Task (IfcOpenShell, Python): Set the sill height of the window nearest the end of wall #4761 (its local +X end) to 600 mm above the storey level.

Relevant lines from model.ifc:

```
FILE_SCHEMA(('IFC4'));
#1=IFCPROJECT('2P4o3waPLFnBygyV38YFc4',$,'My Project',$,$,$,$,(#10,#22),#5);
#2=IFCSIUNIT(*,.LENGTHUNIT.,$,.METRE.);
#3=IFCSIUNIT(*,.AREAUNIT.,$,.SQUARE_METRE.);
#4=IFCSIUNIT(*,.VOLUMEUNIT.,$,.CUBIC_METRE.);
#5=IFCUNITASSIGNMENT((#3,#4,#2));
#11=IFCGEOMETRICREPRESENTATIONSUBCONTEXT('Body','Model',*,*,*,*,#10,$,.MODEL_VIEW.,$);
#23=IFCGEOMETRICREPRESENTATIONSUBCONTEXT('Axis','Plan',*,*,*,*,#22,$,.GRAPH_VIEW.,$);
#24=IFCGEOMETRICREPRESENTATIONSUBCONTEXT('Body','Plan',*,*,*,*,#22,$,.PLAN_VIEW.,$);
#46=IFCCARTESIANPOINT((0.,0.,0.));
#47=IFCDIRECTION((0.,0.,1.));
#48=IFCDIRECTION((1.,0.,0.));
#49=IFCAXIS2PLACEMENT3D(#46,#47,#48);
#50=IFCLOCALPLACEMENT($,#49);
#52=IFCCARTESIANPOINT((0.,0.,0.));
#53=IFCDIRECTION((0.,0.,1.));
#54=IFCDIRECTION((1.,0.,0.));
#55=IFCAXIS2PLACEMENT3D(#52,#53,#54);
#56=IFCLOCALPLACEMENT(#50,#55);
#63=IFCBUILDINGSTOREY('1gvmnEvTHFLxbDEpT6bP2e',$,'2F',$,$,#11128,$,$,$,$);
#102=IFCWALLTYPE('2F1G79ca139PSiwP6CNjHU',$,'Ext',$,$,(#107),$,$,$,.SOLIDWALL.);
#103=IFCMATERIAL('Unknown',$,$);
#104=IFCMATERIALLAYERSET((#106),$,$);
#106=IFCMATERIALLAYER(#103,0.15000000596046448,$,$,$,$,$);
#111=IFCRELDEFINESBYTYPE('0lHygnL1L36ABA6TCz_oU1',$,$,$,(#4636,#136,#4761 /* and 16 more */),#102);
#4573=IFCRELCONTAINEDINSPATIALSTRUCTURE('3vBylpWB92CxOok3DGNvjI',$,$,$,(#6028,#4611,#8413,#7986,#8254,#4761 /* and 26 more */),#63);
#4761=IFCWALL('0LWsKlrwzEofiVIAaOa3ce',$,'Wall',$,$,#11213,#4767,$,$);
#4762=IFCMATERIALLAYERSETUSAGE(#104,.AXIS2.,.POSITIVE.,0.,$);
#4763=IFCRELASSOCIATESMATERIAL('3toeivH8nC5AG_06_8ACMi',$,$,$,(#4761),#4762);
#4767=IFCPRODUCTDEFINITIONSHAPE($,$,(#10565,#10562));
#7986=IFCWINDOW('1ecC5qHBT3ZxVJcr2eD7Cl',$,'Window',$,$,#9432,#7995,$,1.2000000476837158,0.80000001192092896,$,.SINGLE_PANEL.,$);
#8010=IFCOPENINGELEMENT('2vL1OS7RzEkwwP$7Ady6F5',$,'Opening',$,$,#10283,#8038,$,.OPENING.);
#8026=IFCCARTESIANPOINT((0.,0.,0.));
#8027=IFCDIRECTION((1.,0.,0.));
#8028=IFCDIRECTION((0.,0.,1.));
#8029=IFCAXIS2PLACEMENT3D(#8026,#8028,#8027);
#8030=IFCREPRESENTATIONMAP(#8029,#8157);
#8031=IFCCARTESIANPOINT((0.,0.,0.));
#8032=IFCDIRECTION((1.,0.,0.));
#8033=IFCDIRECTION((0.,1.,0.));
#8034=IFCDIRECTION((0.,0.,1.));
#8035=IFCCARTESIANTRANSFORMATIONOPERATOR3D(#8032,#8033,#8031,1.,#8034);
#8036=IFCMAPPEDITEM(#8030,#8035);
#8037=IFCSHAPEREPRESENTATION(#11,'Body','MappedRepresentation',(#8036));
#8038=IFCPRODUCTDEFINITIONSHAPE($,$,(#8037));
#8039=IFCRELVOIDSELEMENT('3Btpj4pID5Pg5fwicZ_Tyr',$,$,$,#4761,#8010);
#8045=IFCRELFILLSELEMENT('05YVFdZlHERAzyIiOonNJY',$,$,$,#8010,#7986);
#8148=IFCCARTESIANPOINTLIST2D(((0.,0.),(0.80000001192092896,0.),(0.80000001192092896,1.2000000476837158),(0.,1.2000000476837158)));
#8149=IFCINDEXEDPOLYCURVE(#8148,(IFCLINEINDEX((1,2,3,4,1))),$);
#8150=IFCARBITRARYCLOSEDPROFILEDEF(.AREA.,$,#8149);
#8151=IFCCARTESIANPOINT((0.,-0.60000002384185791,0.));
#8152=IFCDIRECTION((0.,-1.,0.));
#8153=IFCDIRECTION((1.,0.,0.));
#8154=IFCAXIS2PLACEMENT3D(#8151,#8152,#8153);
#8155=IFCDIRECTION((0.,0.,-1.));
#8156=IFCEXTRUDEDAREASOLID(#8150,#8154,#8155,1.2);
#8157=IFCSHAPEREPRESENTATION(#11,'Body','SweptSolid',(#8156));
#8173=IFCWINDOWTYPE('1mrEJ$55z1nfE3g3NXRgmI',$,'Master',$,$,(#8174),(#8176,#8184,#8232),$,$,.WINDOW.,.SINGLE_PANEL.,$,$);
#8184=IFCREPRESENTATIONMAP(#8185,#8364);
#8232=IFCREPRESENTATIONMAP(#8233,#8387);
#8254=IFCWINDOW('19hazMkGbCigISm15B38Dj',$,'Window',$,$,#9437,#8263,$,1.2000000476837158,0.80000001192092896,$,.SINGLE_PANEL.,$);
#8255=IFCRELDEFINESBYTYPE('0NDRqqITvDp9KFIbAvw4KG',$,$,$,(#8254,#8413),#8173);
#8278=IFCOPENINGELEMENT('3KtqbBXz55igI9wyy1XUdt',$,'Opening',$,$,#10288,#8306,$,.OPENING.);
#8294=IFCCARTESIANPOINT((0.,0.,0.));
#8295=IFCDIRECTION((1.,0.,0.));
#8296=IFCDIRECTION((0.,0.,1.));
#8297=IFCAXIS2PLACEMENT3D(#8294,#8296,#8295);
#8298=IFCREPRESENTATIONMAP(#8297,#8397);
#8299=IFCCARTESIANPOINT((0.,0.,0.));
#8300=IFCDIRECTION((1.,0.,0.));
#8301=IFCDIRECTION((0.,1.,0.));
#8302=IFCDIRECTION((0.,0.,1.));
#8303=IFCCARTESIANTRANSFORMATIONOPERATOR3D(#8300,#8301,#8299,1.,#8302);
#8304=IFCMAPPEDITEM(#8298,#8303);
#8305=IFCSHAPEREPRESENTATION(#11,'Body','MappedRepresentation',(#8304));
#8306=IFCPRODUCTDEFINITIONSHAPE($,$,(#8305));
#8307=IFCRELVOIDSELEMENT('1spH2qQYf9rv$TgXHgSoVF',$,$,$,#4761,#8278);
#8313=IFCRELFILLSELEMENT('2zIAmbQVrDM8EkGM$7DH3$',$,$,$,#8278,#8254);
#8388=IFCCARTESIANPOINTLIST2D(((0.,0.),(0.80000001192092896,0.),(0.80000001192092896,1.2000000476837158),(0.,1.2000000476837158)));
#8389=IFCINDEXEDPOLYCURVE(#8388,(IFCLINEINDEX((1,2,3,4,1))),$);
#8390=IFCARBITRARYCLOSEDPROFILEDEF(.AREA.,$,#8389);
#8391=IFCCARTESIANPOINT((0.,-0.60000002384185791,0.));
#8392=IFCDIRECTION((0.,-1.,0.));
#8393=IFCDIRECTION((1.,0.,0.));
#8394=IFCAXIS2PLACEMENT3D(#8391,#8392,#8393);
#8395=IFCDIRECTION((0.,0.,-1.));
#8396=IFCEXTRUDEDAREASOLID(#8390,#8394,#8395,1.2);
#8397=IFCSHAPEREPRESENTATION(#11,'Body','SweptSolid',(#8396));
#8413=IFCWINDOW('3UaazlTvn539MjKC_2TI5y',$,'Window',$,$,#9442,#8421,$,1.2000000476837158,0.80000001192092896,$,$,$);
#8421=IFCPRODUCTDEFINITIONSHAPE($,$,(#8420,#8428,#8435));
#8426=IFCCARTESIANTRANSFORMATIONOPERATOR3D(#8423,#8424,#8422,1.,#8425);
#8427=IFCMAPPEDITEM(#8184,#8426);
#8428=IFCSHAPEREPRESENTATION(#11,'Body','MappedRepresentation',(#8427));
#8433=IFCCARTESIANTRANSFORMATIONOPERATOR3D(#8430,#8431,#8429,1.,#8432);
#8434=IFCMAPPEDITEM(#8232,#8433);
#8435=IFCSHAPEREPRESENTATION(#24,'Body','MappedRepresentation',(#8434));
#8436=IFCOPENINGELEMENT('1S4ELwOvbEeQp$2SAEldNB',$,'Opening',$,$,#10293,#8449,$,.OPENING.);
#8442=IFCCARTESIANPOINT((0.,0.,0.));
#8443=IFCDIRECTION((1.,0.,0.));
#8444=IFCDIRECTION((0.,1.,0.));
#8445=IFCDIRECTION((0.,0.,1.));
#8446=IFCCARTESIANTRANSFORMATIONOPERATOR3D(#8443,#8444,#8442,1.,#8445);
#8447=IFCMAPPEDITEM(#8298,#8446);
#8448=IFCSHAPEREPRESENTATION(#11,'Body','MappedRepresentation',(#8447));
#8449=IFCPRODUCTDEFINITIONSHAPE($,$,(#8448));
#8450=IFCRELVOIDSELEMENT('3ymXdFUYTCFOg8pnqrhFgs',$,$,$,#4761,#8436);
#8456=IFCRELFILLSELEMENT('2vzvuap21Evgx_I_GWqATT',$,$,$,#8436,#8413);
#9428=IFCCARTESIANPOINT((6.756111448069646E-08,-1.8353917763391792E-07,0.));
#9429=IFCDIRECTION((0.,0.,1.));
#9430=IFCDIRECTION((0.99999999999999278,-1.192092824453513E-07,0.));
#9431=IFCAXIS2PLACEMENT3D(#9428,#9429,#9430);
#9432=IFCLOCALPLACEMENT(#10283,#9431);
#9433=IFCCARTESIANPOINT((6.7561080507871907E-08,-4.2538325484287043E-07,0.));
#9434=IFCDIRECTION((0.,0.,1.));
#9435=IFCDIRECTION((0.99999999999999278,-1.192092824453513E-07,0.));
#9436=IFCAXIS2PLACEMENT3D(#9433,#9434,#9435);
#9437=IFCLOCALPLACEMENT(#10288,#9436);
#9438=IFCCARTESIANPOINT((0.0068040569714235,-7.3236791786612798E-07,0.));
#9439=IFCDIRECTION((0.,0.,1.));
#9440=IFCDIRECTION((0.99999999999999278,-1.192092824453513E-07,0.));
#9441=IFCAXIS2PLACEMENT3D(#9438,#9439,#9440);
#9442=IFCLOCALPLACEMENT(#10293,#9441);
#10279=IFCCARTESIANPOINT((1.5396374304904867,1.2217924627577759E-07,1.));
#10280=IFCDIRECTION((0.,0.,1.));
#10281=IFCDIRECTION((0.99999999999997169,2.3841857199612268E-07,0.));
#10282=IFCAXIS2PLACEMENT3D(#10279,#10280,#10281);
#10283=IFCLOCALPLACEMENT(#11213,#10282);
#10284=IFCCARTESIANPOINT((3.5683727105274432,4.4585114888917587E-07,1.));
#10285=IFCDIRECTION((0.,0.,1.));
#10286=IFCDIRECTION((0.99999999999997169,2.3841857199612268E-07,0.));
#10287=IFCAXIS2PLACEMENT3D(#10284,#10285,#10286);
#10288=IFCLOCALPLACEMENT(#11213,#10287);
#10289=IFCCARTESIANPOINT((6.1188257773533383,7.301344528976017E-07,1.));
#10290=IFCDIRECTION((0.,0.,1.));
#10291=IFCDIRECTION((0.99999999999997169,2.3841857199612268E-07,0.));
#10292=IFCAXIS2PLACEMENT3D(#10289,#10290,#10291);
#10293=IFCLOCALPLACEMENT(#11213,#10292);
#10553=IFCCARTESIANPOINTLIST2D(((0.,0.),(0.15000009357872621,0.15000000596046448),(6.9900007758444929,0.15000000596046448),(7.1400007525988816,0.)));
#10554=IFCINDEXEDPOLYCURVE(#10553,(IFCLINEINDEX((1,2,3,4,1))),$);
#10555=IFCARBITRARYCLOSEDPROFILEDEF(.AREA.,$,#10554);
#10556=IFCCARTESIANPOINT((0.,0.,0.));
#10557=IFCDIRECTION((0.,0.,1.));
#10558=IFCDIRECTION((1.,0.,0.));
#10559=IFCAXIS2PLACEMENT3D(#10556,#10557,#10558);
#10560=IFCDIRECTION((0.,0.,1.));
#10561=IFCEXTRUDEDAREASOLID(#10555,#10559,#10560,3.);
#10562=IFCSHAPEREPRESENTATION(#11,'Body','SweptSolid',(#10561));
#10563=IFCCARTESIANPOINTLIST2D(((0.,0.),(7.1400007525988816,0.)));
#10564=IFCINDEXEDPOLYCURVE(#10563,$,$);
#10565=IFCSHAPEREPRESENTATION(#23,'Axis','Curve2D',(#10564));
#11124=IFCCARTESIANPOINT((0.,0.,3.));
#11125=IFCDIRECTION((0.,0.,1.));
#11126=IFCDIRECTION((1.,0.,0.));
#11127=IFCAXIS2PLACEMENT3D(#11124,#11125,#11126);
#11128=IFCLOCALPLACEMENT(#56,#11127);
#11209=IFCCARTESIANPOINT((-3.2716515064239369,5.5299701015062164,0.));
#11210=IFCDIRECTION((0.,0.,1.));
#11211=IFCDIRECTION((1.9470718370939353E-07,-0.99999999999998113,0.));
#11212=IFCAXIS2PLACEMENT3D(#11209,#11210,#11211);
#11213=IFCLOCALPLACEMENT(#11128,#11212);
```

```python
import numpy as np
import ifcopenshell
import ifcopenshell.api.geometry
import ifcopenshell.geom
import ifcopenshell.util.element
import ifcopenshell.util.placement
import ifcopenshell.util.shape
import ifcopenshell.util.unit

model = ifcopenshell.open("model.ifc")
unit_scale = ifcopenshell.util.unit.calculate_unit_scale(model)

window = model.by_guid("3UaazlTvn539MjKC_2TI5y")
opening = window.FillsVoids[0].RelatingOpeningElement
storey = ifcopenshell.util.element.get_container(window, ifc_class="IfcBuildingStorey")
level = ifcopenshell.util.placement.get_local_placement(storey.ObjectPlacement)[2, 3]

# The opening's origin need not be at the sill, so measure its lowest point.
shape = ifcopenshell.geom.create_shape(ifcopenshell.geom.settings(), opening)
bottom = ifcopenshell.util.shape.get_shape_bottom_elevation(shape, shape.geometry) / unit_scale
dz = level + 0.6 / unit_scale - bottom

shift = np.array([0.0, 0.0, dz])
# The window is placed relative to its opening, so it follows when the opening moves.
matrix = ifcopenshell.util.placement.get_local_placement(opening.ObjectPlacement)
matrix[:3, 3] += shift
ifcopenshell.api.geometry.edit_object_placement(
    model, product=opening, matrix=matrix, is_si=False, should_transform_children=True
)

print(f"moved by {dz * unit_scale:+.3f} m")

model.write("model_edited.ifc")
```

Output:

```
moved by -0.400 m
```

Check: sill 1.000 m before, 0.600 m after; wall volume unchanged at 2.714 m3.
